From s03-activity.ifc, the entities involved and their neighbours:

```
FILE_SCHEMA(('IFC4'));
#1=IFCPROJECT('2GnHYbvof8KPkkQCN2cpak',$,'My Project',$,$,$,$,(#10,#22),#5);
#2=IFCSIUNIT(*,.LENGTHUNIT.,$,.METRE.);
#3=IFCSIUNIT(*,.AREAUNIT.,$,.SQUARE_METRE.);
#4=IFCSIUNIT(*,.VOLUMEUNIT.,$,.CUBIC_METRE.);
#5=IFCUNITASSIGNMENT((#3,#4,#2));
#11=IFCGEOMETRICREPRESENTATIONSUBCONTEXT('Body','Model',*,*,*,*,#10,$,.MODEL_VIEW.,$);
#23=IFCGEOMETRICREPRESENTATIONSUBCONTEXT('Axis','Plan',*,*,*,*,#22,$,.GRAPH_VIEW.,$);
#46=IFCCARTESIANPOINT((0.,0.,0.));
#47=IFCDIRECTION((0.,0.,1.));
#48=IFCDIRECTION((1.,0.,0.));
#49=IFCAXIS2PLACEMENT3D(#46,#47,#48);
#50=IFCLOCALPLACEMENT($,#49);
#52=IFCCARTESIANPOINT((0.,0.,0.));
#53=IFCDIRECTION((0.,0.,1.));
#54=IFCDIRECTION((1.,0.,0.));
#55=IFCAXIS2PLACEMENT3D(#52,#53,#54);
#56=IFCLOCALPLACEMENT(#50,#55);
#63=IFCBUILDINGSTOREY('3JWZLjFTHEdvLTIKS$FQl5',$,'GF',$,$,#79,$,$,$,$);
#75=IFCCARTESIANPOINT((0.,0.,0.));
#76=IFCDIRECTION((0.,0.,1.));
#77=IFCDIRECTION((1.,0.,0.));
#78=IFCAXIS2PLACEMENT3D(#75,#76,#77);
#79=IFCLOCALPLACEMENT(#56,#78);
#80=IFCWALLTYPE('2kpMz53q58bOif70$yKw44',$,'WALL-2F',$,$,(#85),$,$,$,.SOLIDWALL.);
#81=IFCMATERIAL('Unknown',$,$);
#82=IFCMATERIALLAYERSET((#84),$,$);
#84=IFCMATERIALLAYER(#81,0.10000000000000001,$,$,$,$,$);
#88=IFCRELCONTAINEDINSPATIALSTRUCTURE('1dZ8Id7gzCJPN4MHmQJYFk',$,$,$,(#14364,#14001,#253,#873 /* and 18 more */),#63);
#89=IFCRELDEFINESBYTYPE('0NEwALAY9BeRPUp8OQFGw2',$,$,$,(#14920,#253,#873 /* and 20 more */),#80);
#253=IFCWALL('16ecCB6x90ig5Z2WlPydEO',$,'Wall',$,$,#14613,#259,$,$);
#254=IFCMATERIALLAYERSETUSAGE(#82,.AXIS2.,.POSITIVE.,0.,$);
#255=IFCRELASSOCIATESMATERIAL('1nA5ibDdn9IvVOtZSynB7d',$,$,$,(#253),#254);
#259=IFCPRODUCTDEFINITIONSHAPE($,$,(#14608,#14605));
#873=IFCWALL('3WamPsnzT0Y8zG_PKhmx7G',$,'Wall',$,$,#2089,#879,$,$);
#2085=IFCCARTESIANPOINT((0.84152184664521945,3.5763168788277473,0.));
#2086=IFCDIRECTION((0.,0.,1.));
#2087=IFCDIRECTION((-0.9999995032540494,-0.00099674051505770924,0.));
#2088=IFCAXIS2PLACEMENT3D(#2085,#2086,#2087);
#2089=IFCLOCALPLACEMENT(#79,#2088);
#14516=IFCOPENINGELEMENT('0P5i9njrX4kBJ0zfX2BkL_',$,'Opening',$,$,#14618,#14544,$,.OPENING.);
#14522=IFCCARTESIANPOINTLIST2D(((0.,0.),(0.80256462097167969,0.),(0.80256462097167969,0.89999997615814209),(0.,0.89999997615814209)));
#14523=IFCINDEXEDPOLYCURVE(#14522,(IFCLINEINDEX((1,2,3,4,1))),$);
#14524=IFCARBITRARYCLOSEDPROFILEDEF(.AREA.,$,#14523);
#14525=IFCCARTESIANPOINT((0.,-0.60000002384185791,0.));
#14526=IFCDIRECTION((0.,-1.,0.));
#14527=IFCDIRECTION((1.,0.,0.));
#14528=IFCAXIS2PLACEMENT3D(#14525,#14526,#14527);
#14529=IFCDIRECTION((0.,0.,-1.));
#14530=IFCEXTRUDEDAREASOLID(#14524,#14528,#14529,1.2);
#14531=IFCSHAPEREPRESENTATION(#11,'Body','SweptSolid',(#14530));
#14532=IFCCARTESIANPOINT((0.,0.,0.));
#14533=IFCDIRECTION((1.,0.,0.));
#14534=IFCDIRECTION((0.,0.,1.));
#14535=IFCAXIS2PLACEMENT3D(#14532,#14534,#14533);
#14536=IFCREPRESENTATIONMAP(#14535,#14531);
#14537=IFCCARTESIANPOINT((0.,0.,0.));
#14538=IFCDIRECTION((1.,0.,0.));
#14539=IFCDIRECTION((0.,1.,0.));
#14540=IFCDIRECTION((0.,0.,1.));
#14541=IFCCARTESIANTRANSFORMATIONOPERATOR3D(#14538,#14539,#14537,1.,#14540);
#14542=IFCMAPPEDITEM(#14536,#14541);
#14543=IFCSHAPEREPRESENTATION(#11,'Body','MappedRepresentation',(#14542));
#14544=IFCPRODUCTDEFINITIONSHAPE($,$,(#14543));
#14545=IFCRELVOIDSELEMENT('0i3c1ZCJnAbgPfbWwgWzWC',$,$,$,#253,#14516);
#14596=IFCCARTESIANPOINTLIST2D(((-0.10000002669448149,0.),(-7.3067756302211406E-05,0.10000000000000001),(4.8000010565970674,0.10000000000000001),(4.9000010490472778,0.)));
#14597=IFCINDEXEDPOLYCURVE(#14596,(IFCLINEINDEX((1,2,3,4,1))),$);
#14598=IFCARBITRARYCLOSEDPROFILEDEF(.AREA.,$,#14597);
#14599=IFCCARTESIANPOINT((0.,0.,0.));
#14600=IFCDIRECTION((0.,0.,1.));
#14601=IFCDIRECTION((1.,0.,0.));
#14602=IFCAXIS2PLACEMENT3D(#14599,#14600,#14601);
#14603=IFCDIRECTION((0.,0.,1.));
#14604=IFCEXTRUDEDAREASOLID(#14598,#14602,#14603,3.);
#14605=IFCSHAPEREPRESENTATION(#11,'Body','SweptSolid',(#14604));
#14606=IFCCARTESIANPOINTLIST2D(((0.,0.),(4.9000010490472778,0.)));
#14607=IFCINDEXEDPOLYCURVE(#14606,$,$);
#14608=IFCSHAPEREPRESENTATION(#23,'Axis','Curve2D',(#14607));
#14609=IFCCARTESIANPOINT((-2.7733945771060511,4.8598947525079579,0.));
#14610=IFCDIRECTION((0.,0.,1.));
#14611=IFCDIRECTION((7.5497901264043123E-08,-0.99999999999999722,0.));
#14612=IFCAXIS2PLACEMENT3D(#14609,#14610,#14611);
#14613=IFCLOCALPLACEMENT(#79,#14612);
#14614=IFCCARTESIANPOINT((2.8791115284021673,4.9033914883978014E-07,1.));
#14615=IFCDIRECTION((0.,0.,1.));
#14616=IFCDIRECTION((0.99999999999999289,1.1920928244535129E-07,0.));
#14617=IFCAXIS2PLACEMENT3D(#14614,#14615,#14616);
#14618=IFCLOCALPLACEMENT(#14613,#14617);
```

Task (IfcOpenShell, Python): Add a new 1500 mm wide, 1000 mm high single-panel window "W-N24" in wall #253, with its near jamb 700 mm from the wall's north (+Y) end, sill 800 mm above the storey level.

```python
import numpy as np
import ifcopenshell
import ifcopenshell.api.feature
import ifcopenshell.api.geometry
import ifcopenshell.api.root
import ifcopenshell.api.spatial
import ifcopenshell.geom
import ifcopenshell.util.element
import ifcopenshell.util.placement
import ifcopenshell.util.representation
import ifcopenshell.util.shape
import ifcopenshell.util.unit

model = ifcopenshell.open("s03-activity.ifc")
unit_scale = ifcopenshell.util.unit.calculate_unit_scale(model)
settings = ifcopenshell.geom.settings()


def volume(element):
    """Net volume in cubic metres, openings subtracted."""
    shape = ifcopenshell.geom.create_shape(settings, element)
    return ifcopenshell.util.shape.get_volume(shape.geometry)


wall = model.by_guid("16ecCB6x90ig5Z2WlPydEO")
storey = ifcopenshell.util.element.get_container(wall, ifc_class="IfcBuildingStorey")
context = ifcopenshell.util.representation.get_context(model, "Model", "Body", "MODEL_VIEW")
before = volume(wall)

width, height, from_end, sill = 1.5, 1, 0.7, 0.8  # metres

# The wall runs along its own X axis, and the end named is its -X end.
wall_shape = ifcopenshell.geom.create_shape(settings, wall)
x, y, z = ifcopenshell.util.shape.get_vertices(wall_shape.geometry).T
start = x.min() + from_end
face, thickness = float(y.min()), float(y.max() - y.min())
wall_matrix = ifcopenshell.util.placement.get_local_placement(wall.ObjectPlacement)
level = ifcopenshell.util.placement.get_local_placement(storey.ObjectPlacement)[2, 3]


def in_wall(x, y):
    """Placement at x, y metres in the wall's axes, at sill height."""
    matrix = wall_matrix.copy()
    matrix[:, 3] = wall_matrix @ np.array([x / unit_scale, y / unit_scale, 0.0, 1.0])
    matrix[2, 3] = level + sill / unit_scale
    return matrix


# Opening: a box that overshoots both wall faces by 50 mm.
opening = ifcopenshell.api.root.create_entity(model, ifc_class="IfcOpeningElement", predefined_type="OPENING")
box = ifcopenshell.api.geometry.add_wall_representation(
    model, context=context, length=width, height=height, thickness=thickness + 0.1
)
ifcopenshell.api.geometry.assign_representation(model, product=opening, representation=box)
ifcopenshell.api.geometry.edit_object_placement(model, product=opening, matrix=in_wall(start, face - 0.05), is_si=False)
ifcopenshell.api.feature.add_feature(model, feature=opening, element=wall)

window = ifcopenshell.api.root.create_entity(model, ifc_class="IfcWindow", name="W-N24", predefined_type="WINDOW")
window.OverallWidth, window.OverallHeight = width / unit_scale, height / unit_scale
window.PartitioningType = "SINGLE_PANEL"
body = ifcopenshell.api.geometry.add_window_representation(
    model,
    context=context,
    overall_width=window.OverallWidth,
    overall_height=window.OverallHeight,
    partition_type="SINGLE_PANEL",
)
ifcopenshell.api.geometry.assign_representation(model, product=window, representation=body)
ifcopenshell.api.spatial.assign_container(model, products=[window], relating_structure=storey)
ifcopenshell.api.feature.add_filling(model, opening=opening, element=window)

# Centre the window in the wall's thickness.
ifcopenshell.api.geometry.edit_object_placement(model, product=window, matrix=in_wall(start, face), is_si=False)
window_shape = ifcopenshell.geom.create_shape(settings, window)
depth = ifcopenshell.util.shape.get_vertices(window_shape.geometry)[:, 1]
offset = face + thickness / 2 - (depth.min() + depth.max()) / 2
ifcopenshell.api.geometry.edit_object_placement(model, product=window, matrix=in_wall(start, offset), is_si=False)

after = volume(wall)

print(f"wall volume {before:.3f} -> {after:.3f} m3")

model.write("s03-activity_updated.ifc")
```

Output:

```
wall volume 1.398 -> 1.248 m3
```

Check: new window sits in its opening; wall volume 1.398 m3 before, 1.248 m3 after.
